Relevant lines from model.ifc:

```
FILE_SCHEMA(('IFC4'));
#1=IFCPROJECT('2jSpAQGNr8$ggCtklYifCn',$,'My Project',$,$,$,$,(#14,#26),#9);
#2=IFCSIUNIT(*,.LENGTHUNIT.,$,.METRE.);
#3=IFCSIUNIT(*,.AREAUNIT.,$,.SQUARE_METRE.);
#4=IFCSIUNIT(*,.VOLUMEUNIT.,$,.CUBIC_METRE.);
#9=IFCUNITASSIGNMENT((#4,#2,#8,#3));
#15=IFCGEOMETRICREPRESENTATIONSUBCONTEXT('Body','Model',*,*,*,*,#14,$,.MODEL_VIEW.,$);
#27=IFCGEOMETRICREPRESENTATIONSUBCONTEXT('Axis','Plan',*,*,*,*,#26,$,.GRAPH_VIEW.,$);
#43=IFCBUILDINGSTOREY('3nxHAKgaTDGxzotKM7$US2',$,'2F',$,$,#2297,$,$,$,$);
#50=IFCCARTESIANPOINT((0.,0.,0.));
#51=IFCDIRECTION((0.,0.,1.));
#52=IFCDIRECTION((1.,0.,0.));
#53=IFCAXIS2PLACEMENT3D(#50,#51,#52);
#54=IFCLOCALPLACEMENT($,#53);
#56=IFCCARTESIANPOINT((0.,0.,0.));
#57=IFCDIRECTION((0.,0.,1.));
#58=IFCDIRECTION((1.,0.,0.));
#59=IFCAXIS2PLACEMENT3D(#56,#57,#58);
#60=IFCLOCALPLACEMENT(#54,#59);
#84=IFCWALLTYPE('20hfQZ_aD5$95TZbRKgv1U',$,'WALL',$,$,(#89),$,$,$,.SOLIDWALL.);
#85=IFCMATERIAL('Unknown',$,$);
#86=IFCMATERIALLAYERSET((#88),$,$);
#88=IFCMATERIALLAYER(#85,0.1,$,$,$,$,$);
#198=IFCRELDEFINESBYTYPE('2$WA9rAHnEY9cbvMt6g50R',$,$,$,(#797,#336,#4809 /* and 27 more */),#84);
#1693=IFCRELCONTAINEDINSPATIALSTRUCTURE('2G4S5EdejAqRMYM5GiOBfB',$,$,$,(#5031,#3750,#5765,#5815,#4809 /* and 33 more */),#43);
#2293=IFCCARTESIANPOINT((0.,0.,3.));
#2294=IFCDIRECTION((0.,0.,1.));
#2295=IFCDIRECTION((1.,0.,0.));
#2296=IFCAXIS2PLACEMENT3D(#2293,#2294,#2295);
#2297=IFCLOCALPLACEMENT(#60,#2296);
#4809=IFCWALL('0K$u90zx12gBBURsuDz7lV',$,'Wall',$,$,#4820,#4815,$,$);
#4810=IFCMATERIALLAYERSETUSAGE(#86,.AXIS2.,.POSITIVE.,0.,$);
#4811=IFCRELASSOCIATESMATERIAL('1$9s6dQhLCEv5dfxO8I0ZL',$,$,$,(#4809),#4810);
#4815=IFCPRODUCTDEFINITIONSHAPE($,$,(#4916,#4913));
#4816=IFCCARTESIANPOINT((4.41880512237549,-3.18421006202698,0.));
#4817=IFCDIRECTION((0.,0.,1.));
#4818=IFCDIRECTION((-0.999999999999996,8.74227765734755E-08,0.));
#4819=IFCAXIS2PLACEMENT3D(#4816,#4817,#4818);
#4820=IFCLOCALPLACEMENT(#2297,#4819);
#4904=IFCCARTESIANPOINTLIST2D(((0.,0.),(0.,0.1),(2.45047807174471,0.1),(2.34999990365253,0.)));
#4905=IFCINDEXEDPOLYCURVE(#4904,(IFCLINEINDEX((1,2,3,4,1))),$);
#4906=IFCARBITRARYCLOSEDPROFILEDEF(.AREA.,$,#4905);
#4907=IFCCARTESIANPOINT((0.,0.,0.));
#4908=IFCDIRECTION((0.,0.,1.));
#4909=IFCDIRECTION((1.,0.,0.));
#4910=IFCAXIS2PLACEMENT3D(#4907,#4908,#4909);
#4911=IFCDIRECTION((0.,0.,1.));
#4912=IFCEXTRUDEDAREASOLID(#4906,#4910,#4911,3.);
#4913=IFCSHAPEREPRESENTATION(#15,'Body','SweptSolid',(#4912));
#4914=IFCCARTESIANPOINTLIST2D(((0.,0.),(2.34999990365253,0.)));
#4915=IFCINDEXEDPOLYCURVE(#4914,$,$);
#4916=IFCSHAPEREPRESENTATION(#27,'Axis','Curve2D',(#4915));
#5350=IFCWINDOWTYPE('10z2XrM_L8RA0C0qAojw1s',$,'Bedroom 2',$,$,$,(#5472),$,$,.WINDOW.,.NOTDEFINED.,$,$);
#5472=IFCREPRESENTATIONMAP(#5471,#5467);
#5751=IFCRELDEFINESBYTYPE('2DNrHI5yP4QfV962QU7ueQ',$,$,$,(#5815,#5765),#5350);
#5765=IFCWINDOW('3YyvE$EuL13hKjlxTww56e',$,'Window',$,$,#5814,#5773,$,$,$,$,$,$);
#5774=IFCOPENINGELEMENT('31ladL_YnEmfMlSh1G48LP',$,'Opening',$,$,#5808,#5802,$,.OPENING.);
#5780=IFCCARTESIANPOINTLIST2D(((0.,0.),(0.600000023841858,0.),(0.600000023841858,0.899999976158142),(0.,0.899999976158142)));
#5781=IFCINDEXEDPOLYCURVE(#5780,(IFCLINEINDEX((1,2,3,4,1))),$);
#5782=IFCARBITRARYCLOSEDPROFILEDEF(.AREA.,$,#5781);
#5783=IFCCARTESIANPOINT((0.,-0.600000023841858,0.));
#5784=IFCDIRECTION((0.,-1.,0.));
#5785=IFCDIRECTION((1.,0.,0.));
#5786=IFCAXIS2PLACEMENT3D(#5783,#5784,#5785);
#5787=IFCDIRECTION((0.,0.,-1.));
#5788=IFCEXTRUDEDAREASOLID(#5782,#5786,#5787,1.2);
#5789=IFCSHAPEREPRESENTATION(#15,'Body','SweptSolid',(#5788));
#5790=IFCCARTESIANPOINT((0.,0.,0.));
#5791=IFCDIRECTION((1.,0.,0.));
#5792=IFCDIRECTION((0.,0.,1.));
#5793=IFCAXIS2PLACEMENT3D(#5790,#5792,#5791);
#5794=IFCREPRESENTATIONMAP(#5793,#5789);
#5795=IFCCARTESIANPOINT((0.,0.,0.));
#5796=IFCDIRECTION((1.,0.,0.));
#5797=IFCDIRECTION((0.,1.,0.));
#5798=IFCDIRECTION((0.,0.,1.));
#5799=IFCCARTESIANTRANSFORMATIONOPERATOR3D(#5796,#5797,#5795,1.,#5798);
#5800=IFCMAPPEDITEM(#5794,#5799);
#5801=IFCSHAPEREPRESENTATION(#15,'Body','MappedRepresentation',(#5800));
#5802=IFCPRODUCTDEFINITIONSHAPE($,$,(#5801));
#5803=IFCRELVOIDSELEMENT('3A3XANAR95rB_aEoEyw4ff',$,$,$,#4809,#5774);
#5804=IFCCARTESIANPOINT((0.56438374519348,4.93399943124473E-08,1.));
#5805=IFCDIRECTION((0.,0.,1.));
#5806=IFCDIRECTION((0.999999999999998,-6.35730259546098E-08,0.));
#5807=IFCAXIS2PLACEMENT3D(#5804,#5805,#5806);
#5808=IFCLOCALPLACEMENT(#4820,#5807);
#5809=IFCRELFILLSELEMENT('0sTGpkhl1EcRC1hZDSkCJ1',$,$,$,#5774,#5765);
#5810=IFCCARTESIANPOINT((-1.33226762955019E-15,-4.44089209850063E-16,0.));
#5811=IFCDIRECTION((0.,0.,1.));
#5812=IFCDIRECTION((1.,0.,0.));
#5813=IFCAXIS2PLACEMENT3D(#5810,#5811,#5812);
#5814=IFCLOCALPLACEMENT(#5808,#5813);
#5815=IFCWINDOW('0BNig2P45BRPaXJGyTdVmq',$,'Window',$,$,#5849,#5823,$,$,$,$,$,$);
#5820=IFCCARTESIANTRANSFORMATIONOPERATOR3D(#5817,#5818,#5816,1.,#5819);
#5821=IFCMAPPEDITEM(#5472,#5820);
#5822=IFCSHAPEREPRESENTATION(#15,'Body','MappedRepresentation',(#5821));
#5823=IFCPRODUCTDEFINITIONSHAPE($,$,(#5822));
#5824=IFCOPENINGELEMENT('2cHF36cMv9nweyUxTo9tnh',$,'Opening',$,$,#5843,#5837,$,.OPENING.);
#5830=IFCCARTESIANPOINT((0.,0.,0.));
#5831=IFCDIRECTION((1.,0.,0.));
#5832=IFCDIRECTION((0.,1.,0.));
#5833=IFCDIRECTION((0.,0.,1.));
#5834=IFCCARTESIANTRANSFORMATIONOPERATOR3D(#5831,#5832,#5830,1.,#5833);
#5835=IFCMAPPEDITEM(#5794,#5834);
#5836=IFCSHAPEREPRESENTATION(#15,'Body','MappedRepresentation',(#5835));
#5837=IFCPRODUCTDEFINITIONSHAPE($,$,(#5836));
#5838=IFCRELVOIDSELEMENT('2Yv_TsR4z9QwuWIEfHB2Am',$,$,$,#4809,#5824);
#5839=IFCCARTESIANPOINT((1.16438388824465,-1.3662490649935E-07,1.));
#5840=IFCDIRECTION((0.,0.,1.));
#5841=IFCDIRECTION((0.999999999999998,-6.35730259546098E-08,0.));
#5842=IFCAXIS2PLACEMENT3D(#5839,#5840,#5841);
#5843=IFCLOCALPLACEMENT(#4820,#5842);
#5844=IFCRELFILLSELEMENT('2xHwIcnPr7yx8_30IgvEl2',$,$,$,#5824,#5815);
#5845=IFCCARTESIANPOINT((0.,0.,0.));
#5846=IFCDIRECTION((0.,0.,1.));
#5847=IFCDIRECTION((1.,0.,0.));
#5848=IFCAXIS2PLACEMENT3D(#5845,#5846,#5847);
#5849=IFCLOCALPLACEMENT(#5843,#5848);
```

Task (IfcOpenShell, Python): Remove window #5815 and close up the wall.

```python
import ifcopenshell
import ifcopenshell.api.feature
import ifcopenshell.api.root
import ifcopenshell.geom
import ifcopenshell.util.shape

model = ifcopenshell.open("model.ifc")
settings = ifcopenshell.geom.settings()


def volume(element):
    """Net volume in cubic metres, openings subtracted."""
    shape = ifcopenshell.geom.create_shape(settings, element)
    return ifcopenshell.util.shape.get_volume(shape.geometry)


window = model.by_guid("0BNig2P45BRPaXJGyTdVmq")
opening = window.FillsVoids[0].RelatingOpeningElement
wall = opening.VoidsElements[0].RelatingBuildingElement
before = volume(wall)

ifcopenshell.api.root.remove_product(model, product=window)
ifcopenshell.api.feature.remove_feature(model, feature=opening)

after = volume(wall)

print(f"wall volume {before:.3f} -> {after:.3f} m3")

model.write("model_updated.ifc")
```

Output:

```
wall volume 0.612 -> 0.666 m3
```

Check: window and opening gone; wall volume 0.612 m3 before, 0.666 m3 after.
